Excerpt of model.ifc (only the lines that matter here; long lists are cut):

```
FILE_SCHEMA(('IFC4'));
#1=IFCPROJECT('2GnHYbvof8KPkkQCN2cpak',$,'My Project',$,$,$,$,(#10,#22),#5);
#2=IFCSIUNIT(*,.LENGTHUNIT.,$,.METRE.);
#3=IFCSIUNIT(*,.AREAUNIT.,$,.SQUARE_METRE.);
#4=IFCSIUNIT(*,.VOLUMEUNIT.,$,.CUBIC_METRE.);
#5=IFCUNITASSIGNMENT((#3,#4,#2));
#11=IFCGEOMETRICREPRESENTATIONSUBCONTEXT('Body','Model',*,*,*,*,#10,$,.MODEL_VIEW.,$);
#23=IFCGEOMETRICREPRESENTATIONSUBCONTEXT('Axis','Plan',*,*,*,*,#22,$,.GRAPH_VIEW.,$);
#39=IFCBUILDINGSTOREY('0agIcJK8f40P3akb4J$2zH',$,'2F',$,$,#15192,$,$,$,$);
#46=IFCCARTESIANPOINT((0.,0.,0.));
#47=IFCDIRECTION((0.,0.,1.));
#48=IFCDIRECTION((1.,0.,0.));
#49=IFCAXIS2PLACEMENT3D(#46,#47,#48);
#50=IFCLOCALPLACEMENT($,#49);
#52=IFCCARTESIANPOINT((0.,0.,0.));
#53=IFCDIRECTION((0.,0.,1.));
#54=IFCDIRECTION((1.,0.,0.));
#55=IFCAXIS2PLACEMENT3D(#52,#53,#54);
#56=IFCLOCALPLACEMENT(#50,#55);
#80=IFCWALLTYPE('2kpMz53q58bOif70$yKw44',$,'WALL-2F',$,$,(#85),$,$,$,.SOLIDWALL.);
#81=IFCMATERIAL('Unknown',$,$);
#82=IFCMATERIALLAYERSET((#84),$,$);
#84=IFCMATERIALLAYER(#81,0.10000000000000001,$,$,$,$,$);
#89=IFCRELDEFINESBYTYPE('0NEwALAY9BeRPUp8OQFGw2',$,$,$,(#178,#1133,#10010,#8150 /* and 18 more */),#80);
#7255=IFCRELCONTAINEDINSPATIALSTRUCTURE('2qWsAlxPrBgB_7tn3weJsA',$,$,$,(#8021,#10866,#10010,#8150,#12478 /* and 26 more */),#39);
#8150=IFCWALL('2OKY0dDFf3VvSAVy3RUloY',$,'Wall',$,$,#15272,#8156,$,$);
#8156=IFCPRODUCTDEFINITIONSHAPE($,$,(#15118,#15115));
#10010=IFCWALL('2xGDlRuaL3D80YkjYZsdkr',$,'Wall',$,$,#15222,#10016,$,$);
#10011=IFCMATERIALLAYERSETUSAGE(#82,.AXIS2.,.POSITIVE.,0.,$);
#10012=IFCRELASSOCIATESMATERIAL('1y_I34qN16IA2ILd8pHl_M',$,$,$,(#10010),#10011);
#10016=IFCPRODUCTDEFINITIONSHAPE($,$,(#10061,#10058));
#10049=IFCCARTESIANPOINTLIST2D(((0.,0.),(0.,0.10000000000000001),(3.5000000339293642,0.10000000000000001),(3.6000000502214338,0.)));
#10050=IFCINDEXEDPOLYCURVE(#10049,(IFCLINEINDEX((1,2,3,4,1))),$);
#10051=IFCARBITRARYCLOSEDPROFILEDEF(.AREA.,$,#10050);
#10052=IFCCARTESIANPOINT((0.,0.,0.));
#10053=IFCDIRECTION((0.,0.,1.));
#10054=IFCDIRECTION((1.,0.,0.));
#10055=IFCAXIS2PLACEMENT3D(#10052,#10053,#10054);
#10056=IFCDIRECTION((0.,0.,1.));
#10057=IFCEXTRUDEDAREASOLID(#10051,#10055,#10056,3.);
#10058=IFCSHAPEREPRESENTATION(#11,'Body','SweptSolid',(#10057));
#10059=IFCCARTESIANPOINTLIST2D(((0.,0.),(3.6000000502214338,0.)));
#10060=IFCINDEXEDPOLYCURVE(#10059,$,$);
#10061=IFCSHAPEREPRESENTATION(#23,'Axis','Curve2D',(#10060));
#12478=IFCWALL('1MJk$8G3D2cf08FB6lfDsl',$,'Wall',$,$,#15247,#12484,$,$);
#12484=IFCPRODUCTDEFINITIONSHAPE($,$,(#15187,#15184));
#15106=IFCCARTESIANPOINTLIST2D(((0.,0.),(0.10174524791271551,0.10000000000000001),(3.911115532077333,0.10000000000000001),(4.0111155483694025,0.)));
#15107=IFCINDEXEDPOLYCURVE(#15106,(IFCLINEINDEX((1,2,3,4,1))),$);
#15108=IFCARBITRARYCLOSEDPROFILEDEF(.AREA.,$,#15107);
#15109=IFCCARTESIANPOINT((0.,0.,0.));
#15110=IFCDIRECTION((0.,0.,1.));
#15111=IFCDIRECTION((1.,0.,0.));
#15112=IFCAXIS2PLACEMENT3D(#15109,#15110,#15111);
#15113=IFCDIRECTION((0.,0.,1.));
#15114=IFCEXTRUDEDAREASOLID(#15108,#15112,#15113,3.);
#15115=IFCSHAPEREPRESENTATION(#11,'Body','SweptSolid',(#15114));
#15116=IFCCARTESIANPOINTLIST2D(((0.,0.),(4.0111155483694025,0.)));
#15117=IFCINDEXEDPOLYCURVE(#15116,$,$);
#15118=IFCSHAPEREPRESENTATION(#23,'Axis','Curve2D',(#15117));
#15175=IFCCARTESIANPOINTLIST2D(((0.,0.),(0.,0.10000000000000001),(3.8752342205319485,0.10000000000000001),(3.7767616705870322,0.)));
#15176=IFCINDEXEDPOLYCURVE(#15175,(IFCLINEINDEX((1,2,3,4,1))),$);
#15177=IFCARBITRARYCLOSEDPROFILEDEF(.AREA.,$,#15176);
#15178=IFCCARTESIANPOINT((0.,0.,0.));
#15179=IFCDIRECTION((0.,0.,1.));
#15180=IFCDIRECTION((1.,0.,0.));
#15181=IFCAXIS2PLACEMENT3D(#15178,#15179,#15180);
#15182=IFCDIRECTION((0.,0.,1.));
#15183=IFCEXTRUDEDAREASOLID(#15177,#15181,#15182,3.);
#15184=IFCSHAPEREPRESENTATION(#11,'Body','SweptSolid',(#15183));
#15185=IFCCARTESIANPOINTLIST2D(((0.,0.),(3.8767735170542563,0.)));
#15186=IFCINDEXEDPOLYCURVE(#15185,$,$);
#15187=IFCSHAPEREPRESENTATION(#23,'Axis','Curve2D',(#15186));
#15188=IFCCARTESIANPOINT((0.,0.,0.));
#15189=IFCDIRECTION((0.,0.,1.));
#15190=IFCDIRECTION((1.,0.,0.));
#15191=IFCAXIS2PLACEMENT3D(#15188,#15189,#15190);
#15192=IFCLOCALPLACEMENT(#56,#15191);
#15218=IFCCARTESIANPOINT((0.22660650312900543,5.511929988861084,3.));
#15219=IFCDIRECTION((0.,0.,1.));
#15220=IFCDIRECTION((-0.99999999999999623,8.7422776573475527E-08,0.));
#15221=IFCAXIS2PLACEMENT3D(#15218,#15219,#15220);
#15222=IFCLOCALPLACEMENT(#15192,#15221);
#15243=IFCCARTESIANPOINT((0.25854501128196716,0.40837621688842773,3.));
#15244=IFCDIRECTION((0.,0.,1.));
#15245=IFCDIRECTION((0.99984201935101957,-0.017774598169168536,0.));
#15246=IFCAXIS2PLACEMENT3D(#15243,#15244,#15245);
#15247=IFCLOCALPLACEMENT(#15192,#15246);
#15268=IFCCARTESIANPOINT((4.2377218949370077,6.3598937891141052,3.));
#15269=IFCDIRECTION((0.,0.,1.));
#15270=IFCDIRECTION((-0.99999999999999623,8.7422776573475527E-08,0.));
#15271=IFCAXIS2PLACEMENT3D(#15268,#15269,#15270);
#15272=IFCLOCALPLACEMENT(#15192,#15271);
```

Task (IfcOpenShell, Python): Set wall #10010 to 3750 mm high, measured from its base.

```python
import ifcopenshell
import ifcopenshell.geom
import ifcopenshell.util.representation
import ifcopenshell.util.shape
import ifcopenshell.util.unit

model = ifcopenshell.open("model.ifc")
unit_scale = ifcopenshell.util.unit.calculate_unit_scale(model)
settings = ifcopenshell.geom.settings()


def volume(element):
    """Net volume in cubic metres, openings subtracted."""
    shape = ifcopenshell.geom.create_shape(settings, element)
    return ifcopenshell.util.shape.get_volume(shape.geometry)


wall = model.by_id(10010)
before = volume(wall)

body = ifcopenshell.util.representation.get_representation(wall, "Model", "Body")
solid = body.Items[0]
old_height = solid.Depth
solid.Depth = 3.75 / unit_scale
after = volume(wall)

print(f"height {old_height:g} -> {solid.Depth:g}, volume {before:.3f} -> {after:.3f} m3")

model.write("model_v2.ifc")
```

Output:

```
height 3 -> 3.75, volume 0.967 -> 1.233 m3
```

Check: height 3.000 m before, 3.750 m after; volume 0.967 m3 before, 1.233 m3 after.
